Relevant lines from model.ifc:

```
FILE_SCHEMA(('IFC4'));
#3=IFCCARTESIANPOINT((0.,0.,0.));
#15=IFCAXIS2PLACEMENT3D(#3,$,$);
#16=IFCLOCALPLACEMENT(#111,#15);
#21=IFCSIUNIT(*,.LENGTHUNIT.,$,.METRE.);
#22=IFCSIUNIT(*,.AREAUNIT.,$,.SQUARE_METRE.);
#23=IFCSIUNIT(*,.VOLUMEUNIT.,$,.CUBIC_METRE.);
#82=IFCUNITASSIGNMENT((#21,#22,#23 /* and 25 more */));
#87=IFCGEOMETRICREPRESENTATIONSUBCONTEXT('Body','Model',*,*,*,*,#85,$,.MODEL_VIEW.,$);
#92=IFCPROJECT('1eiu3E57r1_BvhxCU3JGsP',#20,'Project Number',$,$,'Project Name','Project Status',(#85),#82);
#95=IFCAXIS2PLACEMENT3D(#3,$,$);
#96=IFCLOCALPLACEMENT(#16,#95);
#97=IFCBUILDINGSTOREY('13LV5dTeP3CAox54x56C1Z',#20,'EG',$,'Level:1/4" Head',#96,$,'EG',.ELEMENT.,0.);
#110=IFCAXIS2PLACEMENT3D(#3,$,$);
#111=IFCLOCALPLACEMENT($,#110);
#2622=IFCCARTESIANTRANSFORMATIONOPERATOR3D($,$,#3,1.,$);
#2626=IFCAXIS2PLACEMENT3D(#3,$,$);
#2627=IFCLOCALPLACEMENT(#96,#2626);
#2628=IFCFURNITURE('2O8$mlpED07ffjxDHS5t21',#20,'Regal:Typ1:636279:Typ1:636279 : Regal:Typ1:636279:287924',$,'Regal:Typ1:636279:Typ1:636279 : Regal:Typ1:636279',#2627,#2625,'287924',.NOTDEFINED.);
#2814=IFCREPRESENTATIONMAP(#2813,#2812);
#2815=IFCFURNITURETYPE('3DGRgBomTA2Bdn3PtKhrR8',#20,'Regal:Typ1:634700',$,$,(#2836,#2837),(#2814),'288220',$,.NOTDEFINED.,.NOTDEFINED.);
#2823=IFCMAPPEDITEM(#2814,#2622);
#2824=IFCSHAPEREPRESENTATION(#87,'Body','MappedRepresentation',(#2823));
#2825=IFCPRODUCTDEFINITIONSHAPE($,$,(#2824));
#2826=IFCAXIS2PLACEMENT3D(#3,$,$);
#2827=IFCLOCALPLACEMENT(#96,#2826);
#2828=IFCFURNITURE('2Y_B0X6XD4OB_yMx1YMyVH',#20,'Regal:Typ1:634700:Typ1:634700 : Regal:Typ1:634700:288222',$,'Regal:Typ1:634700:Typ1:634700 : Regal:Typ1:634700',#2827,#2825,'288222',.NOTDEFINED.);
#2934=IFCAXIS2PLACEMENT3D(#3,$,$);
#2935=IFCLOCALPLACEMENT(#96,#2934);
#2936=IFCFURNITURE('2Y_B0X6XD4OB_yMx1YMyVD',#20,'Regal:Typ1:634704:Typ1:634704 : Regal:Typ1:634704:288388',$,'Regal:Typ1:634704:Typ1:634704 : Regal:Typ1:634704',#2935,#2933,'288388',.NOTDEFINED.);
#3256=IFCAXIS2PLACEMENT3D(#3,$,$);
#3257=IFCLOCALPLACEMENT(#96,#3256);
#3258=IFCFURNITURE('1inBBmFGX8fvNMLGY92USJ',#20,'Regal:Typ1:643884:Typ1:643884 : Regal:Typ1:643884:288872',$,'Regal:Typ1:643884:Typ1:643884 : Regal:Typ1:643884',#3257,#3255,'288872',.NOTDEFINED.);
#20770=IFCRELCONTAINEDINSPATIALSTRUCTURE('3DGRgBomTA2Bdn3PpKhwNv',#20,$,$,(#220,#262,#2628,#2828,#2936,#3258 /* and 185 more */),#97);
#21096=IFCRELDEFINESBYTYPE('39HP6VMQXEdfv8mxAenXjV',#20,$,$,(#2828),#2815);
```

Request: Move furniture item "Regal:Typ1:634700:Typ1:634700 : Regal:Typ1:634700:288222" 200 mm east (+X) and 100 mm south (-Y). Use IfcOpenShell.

```python
import ifcopenshell
import ifcopenshell.api.geometry
import ifcopenshell.util.placement
import ifcopenshell.util.unit

model = ifcopenshell.open("model.ifc")
unit_scale = ifcopenshell.util.unit.calculate_unit_scale(model)

item = model.by_id(2828)
matrix = ifcopenshell.util.placement.get_local_placement(item.ObjectPlacement)
matrix[0, 3] += 0.2 / unit_scale
matrix[1, 3] -= 0.1 / unit_scale
ifcopenshell.api.geometry.edit_object_placement(model, product=item, matrix=matrix, is_si=False)

print(ifcopenshell.util.placement.get_local_placement(item.ObjectPlacement).round(3) + 0.0)

model.write("model_edited.ifc")
```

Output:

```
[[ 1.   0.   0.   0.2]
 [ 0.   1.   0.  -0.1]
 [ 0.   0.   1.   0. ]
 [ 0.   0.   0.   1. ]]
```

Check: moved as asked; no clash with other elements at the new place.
